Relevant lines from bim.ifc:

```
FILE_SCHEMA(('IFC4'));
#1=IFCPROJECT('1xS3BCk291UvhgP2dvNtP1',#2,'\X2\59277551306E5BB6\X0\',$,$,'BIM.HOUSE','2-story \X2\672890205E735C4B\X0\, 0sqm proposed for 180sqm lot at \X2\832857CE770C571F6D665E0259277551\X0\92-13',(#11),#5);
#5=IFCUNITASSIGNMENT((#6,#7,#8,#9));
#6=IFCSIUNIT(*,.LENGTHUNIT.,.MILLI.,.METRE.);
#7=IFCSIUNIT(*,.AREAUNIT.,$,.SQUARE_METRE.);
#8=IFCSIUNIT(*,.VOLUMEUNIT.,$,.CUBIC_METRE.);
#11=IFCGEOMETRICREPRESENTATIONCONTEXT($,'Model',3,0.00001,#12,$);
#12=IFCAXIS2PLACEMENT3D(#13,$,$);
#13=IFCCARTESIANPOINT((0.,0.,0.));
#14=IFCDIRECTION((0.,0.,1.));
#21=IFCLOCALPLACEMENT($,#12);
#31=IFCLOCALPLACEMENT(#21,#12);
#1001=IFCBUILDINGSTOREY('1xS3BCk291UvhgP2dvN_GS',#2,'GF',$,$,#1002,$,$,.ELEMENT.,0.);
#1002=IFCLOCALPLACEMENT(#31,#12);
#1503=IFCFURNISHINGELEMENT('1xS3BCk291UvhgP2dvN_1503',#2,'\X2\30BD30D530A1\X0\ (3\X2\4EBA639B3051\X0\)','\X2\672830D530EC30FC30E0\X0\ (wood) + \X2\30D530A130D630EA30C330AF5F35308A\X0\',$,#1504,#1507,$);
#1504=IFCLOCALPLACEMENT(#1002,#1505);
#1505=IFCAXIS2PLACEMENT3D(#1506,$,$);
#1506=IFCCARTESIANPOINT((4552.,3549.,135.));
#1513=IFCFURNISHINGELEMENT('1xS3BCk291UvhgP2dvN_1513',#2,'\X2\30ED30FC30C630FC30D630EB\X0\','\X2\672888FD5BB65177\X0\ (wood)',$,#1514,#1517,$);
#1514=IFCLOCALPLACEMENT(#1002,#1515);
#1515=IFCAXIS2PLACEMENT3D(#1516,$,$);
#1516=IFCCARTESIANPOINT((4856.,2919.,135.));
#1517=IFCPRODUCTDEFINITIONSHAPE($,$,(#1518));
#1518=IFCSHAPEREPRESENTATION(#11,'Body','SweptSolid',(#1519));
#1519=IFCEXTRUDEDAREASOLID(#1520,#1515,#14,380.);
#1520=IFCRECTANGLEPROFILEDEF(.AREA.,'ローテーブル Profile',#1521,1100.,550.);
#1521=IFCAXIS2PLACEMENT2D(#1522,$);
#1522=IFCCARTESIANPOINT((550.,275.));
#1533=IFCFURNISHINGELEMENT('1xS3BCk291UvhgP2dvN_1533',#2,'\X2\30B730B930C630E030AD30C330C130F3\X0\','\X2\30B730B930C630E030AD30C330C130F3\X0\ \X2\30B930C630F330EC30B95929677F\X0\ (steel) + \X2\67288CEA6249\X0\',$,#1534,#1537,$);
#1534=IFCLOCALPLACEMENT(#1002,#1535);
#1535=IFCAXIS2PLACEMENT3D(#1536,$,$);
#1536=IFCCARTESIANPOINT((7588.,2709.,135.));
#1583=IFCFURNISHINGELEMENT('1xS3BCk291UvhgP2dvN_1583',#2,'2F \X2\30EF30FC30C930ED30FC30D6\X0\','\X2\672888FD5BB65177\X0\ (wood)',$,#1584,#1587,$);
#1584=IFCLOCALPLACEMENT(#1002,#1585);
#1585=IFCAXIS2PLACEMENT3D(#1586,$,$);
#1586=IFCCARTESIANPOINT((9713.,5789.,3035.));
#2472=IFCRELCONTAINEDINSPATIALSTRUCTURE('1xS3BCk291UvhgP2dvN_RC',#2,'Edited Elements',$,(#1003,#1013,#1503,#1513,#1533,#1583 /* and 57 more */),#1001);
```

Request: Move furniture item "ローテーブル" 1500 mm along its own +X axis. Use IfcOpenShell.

```python
import ifcopenshell
import ifcopenshell.api.geometry
import ifcopenshell.util.placement
import ifcopenshell.util.unit

model = ifcopenshell.open("bim.ifc")
unit_scale = ifcopenshell.util.unit.calculate_unit_scale(model)

item = model.by_guid("1xS3BCk291UvhgP2dvN_1513")
matrix = ifcopenshell.util.placement.get_local_placement(item.ObjectPlacement)
matrix[:3, 3] += matrix[:3, 0] * 1.5 / unit_scale
ifcopenshell.api.geometry.edit_object_placement(model, product=item, matrix=matrix, is_si=False)

print(ifcopenshell.util.placement.get_local_placement(item.ObjectPlacement).round(3) + 0.0)

model.write("bim-out.ifc")
```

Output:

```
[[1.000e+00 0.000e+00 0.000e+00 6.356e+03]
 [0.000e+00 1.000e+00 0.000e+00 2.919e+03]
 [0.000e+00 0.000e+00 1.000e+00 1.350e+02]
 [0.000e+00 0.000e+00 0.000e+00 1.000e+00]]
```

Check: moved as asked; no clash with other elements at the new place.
